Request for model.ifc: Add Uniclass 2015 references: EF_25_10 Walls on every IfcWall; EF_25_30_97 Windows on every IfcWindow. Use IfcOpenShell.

First a look at what the model holds.

```python
import ifcopenshell

model = ifcopenshell.open("model.ifc")
print(model.schema)
print("classifications:", [c.Name for c in model.by_type("IfcClassification")])
for ifc_class in ("IfcDoor", "IfcRoof", "IfcStair", "IfcWall", "IfcWindow"):
    print(ifc_class, len(model.by_type(ifc_class)))
```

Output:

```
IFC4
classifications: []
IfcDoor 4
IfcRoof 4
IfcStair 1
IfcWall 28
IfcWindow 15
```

```python
import ifcopenshell
import ifcopenshell.api.classification

model = ifcopenshell.open("model.ifc")

system = ifcopenshell.api.classification.add_classification(model, classification="Uniclass 2015")

codes = {
    "IfcWall": ("EF_25_10", "Walls"),
    "IfcWindow": ("EF_25_30_97", "Windows"),
}
for ifc_class, (code, name) in codes.items():
    products = model.by_type(ifc_class)
    ifcopenshell.api.classification.add_reference(
        model, products=products, classification=system, identification=code, name=name
    )
    print(code, len(products))

model.write("model_v2.ifc")
```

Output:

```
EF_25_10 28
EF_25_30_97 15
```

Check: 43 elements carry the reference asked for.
